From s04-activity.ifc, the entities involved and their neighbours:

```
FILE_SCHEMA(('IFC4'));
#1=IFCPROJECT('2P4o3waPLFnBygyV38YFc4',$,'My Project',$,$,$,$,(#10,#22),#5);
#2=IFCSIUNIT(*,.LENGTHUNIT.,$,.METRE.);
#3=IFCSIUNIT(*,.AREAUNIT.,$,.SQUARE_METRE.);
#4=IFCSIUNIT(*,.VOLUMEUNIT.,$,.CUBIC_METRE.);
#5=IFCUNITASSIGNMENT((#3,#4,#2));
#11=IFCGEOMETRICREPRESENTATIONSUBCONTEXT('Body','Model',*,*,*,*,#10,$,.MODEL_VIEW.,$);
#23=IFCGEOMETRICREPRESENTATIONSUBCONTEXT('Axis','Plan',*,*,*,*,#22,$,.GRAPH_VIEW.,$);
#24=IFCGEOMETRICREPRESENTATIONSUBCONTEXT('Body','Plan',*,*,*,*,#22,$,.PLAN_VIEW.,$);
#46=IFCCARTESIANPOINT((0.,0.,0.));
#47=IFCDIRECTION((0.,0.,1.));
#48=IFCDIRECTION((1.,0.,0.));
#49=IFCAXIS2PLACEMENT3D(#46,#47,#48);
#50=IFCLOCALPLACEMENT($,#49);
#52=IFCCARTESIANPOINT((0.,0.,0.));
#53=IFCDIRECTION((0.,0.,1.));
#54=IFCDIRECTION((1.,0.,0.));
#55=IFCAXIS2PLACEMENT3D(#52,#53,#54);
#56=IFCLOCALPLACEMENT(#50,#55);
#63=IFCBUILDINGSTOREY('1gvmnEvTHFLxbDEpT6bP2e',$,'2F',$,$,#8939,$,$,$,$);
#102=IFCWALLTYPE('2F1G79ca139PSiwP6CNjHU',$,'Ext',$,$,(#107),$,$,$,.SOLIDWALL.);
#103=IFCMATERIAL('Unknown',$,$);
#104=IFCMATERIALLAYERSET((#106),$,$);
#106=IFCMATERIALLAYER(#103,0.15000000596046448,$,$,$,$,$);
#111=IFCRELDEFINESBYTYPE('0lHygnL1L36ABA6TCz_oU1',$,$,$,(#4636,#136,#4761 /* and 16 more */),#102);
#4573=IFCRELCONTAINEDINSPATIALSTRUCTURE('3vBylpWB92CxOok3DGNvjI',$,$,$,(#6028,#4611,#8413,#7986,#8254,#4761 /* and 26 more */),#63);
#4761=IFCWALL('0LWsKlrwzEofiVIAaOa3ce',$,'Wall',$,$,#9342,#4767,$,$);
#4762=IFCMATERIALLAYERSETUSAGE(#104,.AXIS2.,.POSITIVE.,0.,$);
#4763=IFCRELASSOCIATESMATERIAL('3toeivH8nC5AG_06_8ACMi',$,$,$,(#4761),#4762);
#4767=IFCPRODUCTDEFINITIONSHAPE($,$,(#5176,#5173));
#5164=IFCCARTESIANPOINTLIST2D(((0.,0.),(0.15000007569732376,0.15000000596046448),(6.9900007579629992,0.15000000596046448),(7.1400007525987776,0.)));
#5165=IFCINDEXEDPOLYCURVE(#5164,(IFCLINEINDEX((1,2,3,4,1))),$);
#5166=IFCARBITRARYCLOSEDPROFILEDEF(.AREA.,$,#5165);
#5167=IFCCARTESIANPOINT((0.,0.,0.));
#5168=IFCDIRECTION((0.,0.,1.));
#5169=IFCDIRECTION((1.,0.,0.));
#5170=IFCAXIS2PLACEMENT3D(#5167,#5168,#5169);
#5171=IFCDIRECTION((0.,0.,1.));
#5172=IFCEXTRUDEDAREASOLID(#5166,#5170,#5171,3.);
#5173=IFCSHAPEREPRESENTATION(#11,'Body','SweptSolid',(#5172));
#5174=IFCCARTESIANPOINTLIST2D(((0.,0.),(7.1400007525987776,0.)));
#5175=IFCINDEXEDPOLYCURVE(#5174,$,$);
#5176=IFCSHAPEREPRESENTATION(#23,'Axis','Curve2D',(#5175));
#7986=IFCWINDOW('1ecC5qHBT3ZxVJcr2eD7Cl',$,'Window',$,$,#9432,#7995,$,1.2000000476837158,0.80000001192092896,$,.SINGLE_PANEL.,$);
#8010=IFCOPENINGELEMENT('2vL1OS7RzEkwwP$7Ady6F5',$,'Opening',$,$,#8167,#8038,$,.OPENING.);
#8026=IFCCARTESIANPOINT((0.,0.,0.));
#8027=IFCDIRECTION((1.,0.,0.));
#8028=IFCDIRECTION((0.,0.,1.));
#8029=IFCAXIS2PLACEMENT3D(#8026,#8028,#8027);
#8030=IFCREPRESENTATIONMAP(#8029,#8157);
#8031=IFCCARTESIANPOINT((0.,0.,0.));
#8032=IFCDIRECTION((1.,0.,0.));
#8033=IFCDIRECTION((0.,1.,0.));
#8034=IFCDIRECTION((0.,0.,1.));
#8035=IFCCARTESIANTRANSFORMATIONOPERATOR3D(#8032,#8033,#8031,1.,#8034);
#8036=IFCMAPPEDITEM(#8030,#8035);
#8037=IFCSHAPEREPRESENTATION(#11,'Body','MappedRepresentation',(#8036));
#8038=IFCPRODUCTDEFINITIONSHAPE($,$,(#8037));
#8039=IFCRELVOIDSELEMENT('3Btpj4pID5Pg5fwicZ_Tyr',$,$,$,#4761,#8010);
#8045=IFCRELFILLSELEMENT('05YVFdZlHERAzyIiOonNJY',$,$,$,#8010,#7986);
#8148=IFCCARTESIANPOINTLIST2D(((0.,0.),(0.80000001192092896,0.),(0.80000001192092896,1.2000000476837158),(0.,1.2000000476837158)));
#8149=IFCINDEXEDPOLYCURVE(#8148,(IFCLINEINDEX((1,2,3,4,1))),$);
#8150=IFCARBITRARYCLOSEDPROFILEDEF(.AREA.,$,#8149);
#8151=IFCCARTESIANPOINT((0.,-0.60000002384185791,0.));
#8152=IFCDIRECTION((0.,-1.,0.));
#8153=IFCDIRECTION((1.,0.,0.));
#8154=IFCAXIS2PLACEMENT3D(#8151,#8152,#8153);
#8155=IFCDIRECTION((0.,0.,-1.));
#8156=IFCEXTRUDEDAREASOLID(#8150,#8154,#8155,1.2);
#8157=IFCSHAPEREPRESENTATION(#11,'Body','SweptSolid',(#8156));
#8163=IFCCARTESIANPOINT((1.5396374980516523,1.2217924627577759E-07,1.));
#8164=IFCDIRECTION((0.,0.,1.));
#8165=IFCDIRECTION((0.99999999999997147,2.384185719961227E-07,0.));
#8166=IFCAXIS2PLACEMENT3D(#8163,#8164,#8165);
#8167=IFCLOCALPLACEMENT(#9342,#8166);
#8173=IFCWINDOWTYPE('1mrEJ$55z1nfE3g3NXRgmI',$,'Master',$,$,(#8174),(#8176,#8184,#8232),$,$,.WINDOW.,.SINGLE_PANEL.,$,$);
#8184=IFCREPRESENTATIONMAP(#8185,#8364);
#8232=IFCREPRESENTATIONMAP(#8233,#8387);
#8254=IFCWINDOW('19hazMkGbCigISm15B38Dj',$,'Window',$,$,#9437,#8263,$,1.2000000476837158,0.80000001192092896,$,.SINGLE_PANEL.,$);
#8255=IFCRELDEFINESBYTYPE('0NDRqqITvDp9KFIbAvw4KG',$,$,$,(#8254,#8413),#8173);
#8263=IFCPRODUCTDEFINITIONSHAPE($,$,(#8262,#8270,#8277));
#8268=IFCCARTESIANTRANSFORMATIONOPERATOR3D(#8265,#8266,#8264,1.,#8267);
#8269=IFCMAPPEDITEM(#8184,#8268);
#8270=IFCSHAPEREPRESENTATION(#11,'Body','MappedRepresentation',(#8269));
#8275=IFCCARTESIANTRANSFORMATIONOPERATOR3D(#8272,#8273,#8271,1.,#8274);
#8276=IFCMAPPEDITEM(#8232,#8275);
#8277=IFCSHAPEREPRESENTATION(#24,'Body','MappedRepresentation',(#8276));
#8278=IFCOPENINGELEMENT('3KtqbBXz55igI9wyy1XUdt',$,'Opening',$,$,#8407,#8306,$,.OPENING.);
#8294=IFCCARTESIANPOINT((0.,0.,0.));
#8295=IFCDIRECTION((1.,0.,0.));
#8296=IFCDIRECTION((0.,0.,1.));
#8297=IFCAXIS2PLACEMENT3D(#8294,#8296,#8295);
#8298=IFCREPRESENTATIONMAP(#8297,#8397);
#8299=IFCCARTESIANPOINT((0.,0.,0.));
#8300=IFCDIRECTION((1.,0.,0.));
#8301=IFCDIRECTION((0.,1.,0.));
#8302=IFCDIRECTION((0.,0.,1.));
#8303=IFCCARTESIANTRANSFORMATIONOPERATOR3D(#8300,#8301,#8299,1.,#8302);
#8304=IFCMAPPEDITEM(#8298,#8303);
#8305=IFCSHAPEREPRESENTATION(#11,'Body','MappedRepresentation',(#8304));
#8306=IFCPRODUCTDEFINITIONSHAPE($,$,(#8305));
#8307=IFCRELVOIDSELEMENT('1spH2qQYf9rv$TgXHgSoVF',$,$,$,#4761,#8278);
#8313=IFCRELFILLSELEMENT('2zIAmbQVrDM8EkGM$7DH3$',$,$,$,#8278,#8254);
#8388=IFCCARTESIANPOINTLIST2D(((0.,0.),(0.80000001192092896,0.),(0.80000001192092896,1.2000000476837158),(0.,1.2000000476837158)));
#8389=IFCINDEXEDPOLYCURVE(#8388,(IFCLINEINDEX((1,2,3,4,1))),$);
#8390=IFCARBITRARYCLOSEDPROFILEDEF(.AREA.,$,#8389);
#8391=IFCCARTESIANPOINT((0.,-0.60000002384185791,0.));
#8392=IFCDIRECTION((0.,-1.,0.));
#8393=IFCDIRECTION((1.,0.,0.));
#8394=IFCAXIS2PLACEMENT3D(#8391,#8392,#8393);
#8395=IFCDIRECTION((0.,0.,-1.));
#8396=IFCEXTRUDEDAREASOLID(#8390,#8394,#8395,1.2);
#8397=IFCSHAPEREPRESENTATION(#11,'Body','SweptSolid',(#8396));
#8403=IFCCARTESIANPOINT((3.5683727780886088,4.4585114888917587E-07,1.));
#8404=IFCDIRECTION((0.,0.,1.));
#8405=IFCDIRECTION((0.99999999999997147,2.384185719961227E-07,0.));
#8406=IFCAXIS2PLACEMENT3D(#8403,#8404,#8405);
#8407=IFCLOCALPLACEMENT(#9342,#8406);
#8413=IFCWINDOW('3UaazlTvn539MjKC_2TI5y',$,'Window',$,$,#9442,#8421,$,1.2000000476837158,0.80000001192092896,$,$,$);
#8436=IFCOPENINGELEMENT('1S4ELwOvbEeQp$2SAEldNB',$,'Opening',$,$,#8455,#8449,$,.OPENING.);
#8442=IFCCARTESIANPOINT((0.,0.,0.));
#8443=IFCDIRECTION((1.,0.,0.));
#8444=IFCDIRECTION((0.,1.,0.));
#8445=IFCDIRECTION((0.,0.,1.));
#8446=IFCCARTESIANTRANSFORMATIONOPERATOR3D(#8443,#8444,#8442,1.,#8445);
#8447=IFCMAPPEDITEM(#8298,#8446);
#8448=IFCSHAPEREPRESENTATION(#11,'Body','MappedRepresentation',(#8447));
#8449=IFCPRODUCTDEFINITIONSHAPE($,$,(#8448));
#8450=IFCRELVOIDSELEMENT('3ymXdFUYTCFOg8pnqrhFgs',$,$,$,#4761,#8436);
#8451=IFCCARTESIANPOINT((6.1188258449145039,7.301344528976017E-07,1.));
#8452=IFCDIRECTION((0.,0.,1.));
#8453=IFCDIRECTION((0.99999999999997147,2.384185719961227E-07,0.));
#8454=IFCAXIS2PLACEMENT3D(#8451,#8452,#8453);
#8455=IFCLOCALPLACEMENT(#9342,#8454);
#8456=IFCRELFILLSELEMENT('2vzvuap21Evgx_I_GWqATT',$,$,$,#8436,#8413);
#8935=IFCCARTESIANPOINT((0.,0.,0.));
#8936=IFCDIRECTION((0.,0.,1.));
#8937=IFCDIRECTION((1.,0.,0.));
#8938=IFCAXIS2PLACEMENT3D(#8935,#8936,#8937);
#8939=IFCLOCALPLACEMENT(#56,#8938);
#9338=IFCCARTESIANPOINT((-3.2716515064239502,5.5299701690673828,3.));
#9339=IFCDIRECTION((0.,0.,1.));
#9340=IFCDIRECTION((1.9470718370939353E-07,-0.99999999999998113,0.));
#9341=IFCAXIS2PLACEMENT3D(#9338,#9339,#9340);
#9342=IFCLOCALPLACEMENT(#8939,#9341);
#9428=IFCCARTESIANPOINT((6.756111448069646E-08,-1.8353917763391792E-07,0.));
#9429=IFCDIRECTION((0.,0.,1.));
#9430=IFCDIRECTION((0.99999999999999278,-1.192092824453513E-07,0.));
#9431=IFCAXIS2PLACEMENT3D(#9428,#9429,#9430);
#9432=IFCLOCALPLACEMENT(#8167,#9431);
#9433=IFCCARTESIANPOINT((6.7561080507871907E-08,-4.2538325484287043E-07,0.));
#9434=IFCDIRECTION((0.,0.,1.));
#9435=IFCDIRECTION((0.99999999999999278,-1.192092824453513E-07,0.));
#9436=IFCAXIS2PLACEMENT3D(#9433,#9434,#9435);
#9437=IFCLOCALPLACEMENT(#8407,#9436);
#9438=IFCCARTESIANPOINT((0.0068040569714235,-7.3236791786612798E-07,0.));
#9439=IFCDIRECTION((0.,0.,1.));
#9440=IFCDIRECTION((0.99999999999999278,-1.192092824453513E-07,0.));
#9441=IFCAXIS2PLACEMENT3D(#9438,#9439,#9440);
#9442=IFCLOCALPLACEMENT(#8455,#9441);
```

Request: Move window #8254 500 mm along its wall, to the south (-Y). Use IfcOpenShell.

```python
import ifcopenshell
import ifcopenshell.api.geometry
import ifcopenshell.util.placement
import ifcopenshell.util.unit

model = ifcopenshell.open("s04-activity.ifc")
unit_scale = ifcopenshell.util.unit.calculate_unit_scale(model)

window = model.by_guid("19hazMkGbCigISm15B38Dj")
opening = window.FillsVoids[0].RelatingOpeningElement
wall = opening.VoidsElements[0].RelatingBuildingElement

wall_matrix = ifcopenshell.util.placement.get_local_placement(wall.ObjectPlacement)
shift = wall_matrix[:3, 0] * 0.5 / unit_scale
before = ifcopenshell.util.placement.get_local_placement(window.ObjectPlacement)[:3, 3].copy()

# The window is placed relative to its opening, so it follows when the opening moves.
matrix = ifcopenshell.util.placement.get_local_placement(opening.ObjectPlacement)
matrix[:3, 3] += shift
ifcopenshell.api.geometry.edit_object_placement(
    model, product=opening, matrix=matrix, is_si=False, should_transform_children=True
)

after = ifcopenshell.util.placement.get_local_placement(window.ObjectPlacement)[:3, 3]
print("window moved by", (after - before).round(3) + 0.0)

model.write("s04-activity_rev.ifc")
```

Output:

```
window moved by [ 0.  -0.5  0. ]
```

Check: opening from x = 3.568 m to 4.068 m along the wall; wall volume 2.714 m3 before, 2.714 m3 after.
